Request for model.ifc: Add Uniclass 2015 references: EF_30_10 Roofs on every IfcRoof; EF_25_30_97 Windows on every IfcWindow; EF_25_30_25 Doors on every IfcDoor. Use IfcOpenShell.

First a look at what the model holds.

```python
import ifcopenshell

model = ifcopenshell.open("model.ifc")
print(model.schema)
print("classifications:", [c.Name for c in model.by_type("IfcClassification")])
for ifc_class in ("IfcDoor", "IfcRoof", "IfcStair", "IfcWall", "IfcWindow"):
    print(ifc_class, len(model.by_type(ifc_class)))
```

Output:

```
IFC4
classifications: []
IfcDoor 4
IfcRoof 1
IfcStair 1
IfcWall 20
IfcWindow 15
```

```python
import ifcopenshell
import ifcopenshell.api.classification

model = ifcopenshell.open("model.ifc")

system = ifcopenshell.api.classification.add_classification(model, classification="Uniclass 2015")

codes = {
    "IfcRoof": ("EF_30_10", "Roofs"),
    "IfcWindow": ("EF_25_30_97", "Windows"),
    "IfcDoor": ("EF_25_30_25", "Doors"),
}
for ifc_class, (code, name) in codes.items():
    products = model.by_type(ifc_class)
    ifcopenshell.api.classification.add_reference(
        model, products=products, classification=system, identification=code, name=name
    )
    print(code, len(products))

model.write("model_edited.ifc")
```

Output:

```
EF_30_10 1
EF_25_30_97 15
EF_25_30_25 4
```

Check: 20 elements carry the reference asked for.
